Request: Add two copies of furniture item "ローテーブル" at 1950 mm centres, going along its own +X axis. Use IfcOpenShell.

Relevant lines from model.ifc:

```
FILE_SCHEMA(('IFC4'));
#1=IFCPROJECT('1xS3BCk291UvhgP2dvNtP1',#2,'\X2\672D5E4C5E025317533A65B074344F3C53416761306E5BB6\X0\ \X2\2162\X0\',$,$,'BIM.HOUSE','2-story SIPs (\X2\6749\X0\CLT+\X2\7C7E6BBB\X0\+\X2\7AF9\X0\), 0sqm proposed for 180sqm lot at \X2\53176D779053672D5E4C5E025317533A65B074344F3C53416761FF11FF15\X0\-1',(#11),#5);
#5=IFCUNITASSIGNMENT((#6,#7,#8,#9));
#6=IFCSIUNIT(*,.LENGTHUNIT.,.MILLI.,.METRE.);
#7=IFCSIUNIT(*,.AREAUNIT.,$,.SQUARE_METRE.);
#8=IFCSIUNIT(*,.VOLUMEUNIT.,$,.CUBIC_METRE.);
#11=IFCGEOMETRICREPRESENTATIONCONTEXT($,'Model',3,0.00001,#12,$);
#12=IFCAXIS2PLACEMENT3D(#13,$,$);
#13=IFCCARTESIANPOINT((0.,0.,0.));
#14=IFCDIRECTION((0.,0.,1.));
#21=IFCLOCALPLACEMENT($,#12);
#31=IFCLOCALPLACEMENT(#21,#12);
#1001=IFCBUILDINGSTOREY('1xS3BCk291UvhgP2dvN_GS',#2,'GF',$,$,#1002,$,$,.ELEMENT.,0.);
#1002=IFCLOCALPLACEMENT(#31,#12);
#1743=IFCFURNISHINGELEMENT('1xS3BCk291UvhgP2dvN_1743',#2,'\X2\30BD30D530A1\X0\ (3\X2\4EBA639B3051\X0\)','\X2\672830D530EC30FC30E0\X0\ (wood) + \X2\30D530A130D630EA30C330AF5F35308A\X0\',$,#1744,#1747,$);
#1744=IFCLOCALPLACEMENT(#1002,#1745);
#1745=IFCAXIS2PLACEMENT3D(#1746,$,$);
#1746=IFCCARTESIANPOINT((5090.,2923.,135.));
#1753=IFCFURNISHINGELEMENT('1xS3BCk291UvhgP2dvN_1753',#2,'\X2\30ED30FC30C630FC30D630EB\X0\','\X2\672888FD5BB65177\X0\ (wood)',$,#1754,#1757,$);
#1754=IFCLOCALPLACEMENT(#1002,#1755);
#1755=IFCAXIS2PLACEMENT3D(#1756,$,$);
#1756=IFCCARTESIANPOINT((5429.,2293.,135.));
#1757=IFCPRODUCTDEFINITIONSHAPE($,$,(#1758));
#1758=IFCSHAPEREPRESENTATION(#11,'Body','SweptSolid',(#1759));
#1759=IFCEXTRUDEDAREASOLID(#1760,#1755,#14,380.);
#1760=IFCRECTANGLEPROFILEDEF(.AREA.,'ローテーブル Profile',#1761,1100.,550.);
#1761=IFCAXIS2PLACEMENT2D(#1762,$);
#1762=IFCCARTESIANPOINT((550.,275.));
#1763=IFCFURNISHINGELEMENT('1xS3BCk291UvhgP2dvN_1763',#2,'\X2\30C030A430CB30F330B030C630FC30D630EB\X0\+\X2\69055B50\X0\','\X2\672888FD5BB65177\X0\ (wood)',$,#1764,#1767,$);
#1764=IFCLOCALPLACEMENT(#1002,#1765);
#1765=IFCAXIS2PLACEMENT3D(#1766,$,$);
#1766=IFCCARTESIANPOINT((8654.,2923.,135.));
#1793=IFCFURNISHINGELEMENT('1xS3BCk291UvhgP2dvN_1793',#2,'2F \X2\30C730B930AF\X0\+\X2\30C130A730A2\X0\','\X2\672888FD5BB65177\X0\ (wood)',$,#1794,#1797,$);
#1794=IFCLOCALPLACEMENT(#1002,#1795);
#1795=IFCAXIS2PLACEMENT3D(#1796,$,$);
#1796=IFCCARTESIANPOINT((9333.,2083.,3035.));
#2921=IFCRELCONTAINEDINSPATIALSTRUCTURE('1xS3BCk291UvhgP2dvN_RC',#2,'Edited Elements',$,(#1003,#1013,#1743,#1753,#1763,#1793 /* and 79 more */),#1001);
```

```python
import ifcopenshell
import ifcopenshell.api.geometry
import ifcopenshell.api.root
import ifcopenshell.util.element
import ifcopenshell.util.placement
import ifcopenshell.util.unit

model = ifcopenshell.open("model.ifc")
unit_scale = ifcopenshell.util.unit.calculate_unit_scale(model)


def reuse_history(source, copy):
    """copy_class also copies each property set's owner history, people and application; keep the originals."""
    for rel in copy.IsDefinedBy:
        if rel.is_a("IfcRelDefinesByProperties") and (history := rel.RelatingPropertyDefinition.OwnerHistory):
            rel.RelatingPropertyDefinition.OwnerHistory = source.OwnerHistory
            ifcopenshell.util.element.remove_deep2(model, history)


source = model.by_guid("1xS3BCk291UvhgP2dvN_1753")
base = ifcopenshell.util.placement.get_local_placement(source.ObjectPlacement)
step = base[:3, 0] * 1.95 / unit_scale

for i in range(1, 3):
    copy = ifcopenshell.api.root.copy_class(model, product=source)
    copy.Representation = ifcopenshell.util.element.copy_deep(
        model, source.Representation, exclude=["IfcGeometricRepresentationContext", "IfcRepresentationMap"]
    )
    reuse_history(source, copy)
    matrix = base.copy()
    matrix[:3, 3] += i * step
    print("added at", matrix[:3, 3].round(3) + 0.0)
    ifcopenshell.api.geometry.edit_object_placement(model, product=copy, matrix=matrix, is_si=False)

model.write("model_updated.ifc")
```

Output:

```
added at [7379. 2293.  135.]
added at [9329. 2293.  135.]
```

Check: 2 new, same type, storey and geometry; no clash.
